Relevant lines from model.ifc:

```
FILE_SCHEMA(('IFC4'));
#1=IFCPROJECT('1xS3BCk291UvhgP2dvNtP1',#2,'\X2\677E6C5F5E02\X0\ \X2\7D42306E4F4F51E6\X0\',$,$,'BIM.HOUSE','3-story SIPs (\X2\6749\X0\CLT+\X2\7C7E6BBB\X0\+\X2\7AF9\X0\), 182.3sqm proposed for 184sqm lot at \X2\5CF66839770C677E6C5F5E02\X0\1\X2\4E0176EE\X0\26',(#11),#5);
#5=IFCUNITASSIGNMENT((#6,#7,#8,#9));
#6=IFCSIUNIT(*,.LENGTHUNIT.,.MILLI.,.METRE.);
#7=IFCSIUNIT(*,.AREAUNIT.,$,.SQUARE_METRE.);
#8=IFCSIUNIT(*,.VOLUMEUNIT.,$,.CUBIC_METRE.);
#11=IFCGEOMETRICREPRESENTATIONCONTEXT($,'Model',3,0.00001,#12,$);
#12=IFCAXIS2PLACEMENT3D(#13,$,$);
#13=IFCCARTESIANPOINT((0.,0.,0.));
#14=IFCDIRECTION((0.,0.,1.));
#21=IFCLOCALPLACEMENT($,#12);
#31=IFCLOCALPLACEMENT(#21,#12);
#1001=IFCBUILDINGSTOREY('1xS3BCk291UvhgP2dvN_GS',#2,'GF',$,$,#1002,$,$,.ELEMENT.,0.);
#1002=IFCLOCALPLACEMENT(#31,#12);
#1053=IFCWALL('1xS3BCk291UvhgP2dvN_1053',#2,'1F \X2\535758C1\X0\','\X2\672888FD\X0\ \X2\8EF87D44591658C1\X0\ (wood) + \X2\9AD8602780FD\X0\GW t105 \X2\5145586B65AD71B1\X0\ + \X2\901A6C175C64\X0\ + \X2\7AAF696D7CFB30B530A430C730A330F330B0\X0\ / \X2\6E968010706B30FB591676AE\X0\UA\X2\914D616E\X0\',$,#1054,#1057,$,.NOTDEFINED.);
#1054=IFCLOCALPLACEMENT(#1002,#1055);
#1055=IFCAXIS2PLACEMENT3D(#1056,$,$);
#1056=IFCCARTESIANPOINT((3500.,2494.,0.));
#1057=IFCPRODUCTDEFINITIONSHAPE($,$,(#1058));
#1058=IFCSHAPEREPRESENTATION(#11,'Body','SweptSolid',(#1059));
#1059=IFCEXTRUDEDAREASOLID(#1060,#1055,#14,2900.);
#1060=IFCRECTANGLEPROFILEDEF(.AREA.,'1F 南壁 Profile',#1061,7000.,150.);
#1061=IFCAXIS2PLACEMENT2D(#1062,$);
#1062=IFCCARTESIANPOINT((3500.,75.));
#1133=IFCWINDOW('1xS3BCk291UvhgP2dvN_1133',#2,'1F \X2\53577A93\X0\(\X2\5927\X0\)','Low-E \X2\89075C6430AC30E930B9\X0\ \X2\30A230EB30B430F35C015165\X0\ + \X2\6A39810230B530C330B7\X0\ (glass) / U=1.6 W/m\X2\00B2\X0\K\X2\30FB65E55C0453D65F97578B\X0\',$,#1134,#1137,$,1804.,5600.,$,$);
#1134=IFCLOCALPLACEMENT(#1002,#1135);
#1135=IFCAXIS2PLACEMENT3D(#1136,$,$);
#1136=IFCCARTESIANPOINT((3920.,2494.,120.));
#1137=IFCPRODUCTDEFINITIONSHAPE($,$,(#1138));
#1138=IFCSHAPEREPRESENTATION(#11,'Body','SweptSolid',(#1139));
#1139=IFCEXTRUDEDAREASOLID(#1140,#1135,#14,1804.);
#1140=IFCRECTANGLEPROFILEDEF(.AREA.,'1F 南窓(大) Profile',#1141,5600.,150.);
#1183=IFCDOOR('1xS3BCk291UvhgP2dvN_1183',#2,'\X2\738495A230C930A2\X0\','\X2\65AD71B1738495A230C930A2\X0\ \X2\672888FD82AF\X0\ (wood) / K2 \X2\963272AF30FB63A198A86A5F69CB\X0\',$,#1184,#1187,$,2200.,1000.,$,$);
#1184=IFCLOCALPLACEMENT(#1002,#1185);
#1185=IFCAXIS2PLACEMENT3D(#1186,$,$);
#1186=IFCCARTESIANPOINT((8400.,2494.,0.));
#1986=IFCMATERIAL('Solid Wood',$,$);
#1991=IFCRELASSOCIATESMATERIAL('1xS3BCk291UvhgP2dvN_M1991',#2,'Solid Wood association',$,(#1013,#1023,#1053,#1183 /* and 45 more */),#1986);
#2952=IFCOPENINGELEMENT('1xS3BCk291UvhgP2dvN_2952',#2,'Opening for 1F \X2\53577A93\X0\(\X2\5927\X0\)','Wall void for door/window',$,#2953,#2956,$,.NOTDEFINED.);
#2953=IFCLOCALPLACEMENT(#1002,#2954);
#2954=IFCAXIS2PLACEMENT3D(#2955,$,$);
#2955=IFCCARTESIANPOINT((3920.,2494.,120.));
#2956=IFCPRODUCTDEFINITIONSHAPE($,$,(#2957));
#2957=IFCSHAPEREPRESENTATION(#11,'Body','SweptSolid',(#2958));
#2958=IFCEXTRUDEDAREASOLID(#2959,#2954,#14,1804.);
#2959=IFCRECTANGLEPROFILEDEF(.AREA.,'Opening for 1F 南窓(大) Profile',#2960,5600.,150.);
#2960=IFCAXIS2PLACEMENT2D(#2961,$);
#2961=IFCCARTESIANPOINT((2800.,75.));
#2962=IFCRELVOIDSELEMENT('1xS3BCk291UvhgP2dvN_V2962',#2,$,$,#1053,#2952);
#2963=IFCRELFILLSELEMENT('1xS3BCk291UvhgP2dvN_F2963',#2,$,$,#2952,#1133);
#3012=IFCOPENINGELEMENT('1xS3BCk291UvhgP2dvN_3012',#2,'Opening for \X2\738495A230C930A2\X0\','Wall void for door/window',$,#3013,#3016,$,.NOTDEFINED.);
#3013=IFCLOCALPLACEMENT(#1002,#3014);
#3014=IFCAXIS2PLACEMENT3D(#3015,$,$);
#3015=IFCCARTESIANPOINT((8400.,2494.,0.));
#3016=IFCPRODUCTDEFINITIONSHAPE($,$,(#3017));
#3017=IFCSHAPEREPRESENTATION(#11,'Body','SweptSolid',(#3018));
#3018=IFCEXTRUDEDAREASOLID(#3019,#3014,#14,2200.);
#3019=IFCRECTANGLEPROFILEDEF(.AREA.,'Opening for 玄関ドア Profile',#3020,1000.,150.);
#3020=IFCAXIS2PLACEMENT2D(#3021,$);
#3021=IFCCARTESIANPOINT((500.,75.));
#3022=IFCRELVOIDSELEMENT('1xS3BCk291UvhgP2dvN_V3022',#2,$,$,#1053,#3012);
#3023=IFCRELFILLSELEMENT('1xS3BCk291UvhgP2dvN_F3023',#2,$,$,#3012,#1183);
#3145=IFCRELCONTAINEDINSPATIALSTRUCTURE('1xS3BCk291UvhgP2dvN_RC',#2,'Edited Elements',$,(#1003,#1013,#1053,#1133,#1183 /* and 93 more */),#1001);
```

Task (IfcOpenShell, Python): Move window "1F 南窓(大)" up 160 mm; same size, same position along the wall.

```python
import numpy as np
import ifcopenshell
import ifcopenshell.api.geometry
import ifcopenshell.util.placement
import ifcopenshell.util.unit

model = ifcopenshell.open("model.ifc")
unit_scale = ifcopenshell.util.unit.calculate_unit_scale(model)

window = model.by_id(1133)
opening = window.FillsVoids[0].RelatingOpeningElement
dz = 0.16 / unit_scale

shift = np.array([0.0, 0.0, dz])
# The window is not placed relative to its opening, so move both.
for product in (opening, window):
    matrix = ifcopenshell.util.placement.get_local_placement(product.ObjectPlacement)
    matrix[:3, 3] += shift
    ifcopenshell.api.geometry.edit_object_placement(model, product=product, matrix=matrix, is_si=False)

print(f"moved by {dz * unit_scale:+.3f} m")

model.write("model_v2.ifc")
```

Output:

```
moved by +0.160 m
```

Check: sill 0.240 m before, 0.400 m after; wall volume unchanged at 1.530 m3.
